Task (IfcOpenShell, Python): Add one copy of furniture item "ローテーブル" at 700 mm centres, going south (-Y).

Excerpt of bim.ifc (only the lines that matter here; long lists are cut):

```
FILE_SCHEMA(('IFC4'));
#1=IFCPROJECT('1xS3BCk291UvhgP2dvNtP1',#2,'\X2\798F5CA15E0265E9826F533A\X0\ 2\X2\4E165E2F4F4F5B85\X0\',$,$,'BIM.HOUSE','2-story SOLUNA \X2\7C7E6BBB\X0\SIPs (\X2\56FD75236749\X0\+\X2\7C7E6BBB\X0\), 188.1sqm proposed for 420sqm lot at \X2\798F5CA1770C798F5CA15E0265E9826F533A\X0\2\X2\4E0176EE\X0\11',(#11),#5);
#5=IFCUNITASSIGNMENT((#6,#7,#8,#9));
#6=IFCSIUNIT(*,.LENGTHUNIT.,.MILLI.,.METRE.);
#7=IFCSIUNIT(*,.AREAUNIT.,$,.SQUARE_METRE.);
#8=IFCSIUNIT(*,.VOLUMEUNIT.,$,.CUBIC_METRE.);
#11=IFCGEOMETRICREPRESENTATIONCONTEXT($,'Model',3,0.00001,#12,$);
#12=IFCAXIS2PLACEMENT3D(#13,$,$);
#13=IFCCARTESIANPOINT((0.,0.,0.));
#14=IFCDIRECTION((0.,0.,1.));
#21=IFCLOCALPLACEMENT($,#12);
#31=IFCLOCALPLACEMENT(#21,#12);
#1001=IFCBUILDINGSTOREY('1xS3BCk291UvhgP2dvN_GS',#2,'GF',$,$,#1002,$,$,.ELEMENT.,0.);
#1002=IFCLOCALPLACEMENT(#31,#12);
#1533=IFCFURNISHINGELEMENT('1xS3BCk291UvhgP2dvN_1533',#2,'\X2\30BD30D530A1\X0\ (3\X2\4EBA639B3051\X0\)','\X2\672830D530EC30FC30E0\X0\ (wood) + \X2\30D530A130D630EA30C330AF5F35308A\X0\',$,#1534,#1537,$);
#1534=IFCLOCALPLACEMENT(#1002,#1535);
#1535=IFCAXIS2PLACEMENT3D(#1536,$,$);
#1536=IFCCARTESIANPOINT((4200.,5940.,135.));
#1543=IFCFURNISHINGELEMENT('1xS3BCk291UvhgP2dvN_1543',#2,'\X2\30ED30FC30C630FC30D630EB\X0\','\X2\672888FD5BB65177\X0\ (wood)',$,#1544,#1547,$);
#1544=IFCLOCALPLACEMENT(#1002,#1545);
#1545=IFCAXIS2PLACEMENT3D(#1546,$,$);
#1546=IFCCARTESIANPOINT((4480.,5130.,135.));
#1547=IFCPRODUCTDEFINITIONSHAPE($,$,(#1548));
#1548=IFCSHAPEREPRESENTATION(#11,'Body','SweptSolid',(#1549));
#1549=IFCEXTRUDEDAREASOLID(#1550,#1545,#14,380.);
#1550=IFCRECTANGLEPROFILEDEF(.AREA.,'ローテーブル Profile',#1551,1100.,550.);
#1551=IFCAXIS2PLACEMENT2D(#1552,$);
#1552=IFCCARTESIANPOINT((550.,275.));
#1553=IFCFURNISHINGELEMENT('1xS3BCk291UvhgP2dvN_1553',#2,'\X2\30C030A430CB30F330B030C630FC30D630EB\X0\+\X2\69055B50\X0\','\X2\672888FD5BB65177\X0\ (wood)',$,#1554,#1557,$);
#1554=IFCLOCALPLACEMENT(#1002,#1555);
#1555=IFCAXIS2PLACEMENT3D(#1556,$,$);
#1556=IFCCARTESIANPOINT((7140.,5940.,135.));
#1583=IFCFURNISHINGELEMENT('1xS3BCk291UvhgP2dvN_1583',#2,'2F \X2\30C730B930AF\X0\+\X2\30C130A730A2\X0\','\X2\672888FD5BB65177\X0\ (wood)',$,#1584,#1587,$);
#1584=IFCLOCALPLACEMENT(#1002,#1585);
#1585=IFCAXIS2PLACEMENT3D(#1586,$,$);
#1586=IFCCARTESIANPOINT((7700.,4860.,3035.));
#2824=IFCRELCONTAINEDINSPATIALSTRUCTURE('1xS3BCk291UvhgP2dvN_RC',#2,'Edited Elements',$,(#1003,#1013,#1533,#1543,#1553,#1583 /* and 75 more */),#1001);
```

```python
import numpy as np
import ifcopenshell
import ifcopenshell.api.geometry
import ifcopenshell.api.root
import ifcopenshell.util.element
import ifcopenshell.util.placement

model = ifcopenshell.open("bim.ifc")


def reuse_history(source, copy):
    """copy_class also copies each property set's owner history, people and application; keep the originals."""
    for rel in copy.IsDefinedBy:
        if rel.is_a("IfcRelDefinesByProperties") and (history := rel.RelatingPropertyDefinition.OwnerHistory):
            rel.RelatingPropertyDefinition.OwnerHistory = source.OwnerHistory
            ifcopenshell.util.element.remove_deep2(model, history)


source = model.by_guid("1xS3BCk291UvhgP2dvN_1543")
base = ifcopenshell.util.placement.get_local_placement(source.ObjectPlacement)
step = np.array([0.0, -1.0, 0.0]) * 700.0

for i in range(1, 2):
    copy = ifcopenshell.api.root.copy_class(model, product=source)
    copy.Representation = ifcopenshell.util.element.copy_deep(
        model, source.Representation, exclude=["IfcGeometricRepresentationContext", "IfcRepresentationMap"]
    )
    reuse_history(source, copy)
    matrix = base.copy()
    matrix[:3, 3] += i * step
    print("added at", matrix[:3, 3].round(3) + 0.0)
    ifcopenshell.api.geometry.edit_object_placement(model, product=copy, matrix=matrix, is_si=False)

model.write("bim_v2.ifc")
```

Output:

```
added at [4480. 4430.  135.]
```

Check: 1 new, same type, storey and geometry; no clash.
